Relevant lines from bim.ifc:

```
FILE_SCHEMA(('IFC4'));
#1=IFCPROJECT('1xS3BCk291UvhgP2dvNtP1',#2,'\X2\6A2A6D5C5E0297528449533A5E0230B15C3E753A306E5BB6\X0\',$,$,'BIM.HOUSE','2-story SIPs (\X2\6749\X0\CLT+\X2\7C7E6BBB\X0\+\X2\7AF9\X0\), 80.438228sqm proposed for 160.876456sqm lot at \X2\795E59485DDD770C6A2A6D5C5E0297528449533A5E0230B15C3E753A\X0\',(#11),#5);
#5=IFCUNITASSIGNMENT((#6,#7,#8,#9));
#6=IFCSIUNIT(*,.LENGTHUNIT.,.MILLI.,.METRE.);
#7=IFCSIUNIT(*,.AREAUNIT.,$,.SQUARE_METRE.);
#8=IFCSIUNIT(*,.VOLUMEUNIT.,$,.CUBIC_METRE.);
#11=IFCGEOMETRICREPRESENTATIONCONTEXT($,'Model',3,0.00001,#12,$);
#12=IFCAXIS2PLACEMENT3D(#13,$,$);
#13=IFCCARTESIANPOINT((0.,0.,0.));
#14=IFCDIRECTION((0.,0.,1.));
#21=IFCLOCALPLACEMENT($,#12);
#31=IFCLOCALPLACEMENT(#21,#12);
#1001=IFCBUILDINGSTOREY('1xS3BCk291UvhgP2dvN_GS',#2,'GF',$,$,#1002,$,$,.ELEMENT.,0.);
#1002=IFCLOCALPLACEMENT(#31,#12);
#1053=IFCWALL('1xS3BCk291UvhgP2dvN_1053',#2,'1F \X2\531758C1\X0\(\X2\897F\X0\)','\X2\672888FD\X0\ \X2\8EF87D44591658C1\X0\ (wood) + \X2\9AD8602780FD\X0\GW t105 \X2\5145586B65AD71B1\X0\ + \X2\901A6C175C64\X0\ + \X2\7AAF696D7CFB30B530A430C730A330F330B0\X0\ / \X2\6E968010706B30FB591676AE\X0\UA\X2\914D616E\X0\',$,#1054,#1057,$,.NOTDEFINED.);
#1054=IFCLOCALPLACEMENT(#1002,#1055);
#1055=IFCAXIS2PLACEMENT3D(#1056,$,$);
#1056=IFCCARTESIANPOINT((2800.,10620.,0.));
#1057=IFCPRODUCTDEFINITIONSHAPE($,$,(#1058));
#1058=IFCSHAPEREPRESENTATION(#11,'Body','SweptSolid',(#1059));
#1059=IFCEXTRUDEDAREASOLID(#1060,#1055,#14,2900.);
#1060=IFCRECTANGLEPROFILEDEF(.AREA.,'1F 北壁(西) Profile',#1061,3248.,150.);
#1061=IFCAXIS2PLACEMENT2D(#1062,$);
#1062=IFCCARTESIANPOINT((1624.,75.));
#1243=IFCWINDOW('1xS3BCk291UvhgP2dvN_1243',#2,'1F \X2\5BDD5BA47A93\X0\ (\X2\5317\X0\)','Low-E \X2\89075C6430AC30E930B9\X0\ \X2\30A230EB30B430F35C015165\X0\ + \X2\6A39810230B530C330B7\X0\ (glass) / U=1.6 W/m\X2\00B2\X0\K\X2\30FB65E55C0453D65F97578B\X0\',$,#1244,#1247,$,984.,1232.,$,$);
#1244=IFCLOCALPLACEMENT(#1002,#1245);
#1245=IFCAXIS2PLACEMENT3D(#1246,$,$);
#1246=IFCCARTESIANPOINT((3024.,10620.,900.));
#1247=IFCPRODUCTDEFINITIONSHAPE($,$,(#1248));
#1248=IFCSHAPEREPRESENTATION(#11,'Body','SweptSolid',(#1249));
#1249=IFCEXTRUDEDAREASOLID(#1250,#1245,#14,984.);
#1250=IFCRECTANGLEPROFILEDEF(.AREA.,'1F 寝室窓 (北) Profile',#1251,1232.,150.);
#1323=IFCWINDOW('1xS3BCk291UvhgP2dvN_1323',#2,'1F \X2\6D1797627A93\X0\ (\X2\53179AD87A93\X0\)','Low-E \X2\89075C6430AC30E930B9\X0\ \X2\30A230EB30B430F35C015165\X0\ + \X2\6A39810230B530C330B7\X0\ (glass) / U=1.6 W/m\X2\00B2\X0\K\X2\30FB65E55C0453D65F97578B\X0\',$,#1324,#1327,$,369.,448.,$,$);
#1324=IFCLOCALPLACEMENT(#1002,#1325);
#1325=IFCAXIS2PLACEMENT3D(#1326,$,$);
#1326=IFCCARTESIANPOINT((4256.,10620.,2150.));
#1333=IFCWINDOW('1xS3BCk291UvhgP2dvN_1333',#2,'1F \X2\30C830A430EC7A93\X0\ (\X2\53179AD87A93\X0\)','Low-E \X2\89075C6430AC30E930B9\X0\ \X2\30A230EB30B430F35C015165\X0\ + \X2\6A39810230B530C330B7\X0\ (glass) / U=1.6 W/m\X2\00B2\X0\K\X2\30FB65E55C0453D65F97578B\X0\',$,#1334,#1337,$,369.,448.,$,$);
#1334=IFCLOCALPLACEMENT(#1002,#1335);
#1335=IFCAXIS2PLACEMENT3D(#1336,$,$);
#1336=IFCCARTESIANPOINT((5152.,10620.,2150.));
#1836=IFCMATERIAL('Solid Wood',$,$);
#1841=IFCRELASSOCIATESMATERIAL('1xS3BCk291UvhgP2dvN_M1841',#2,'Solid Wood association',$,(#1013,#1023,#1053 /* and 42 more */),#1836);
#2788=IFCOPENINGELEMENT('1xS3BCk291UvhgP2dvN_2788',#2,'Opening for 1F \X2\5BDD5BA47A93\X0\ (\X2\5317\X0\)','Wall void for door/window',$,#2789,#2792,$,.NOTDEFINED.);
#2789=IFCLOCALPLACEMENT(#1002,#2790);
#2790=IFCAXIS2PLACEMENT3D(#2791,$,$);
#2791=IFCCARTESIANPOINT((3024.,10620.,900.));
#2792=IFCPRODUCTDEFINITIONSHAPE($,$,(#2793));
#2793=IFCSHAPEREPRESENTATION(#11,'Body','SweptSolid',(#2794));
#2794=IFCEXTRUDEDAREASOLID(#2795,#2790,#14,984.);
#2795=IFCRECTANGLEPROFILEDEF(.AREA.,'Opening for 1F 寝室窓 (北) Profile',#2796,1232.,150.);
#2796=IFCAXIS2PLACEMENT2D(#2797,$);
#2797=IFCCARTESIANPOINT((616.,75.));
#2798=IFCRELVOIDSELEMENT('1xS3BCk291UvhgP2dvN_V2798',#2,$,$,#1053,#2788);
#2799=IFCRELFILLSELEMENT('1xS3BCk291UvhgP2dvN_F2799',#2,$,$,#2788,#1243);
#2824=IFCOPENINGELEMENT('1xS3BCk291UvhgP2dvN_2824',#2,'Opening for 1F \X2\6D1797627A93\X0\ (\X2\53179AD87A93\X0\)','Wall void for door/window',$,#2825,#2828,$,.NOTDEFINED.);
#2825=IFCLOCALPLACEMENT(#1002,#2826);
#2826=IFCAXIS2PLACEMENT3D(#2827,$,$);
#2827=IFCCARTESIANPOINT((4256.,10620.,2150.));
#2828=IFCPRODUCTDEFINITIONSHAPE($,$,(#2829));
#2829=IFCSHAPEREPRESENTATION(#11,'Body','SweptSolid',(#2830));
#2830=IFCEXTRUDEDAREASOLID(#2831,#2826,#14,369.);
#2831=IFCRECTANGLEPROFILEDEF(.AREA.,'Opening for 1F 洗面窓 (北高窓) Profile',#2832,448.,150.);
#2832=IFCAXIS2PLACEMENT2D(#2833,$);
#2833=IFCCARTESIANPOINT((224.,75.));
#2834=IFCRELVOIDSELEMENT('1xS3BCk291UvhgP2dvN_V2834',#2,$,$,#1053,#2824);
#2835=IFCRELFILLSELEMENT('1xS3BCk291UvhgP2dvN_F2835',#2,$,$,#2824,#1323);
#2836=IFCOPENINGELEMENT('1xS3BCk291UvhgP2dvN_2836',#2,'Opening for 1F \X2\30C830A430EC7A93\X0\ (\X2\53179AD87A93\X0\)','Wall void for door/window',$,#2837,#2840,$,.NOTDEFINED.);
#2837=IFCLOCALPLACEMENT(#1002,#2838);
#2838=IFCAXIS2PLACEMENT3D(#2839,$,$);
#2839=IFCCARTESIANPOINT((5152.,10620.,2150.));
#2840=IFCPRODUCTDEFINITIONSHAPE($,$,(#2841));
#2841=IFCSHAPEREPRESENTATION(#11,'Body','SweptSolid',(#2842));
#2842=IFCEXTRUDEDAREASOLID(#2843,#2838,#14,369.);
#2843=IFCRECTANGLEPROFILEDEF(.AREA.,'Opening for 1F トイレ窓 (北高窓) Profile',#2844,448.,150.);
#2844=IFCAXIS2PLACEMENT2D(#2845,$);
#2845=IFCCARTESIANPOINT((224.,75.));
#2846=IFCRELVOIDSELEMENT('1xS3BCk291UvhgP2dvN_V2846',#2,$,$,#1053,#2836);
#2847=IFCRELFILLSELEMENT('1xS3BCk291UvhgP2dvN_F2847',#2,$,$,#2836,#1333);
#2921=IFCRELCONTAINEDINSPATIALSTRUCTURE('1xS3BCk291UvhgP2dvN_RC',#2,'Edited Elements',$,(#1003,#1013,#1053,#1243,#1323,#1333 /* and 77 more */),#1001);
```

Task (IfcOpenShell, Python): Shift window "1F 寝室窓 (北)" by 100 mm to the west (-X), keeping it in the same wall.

```python
import ifcopenshell
import ifcopenshell.api.geometry
import ifcopenshell.util.placement
import ifcopenshell.util.unit

model = ifcopenshell.open("bim.ifc")
unit_scale = ifcopenshell.util.unit.calculate_unit_scale(model)

window = model.by_guid("1xS3BCk291UvhgP2dvN_1243")
opening = window.FillsVoids[0].RelatingOpeningElement
wall = opening.VoidsElements[0].RelatingBuildingElement

wall_matrix = ifcopenshell.util.placement.get_local_placement(wall.ObjectPlacement)
shift = wall_matrix[:3, 0] * -0.1 / unit_scale
before = ifcopenshell.util.placement.get_local_placement(window.ObjectPlacement)[:3, 3].copy()

# The window is not placed relative to its opening, so move both.
for product in (opening, window):
    matrix = ifcopenshell.util.placement.get_local_placement(product.ObjectPlacement)
    matrix[:3, 3] += shift
    ifcopenshell.api.geometry.edit_object_placement(model, product=product, matrix=matrix, is_si=False)

after = ifcopenshell.util.placement.get_local_placement(window.ObjectPlacement)[:3, 3]
print("window moved by", (after - before).round(3) + 0.0)

model.write("bim-out.ifc")
```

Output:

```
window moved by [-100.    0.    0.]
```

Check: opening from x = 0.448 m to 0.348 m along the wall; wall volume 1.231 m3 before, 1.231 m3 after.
